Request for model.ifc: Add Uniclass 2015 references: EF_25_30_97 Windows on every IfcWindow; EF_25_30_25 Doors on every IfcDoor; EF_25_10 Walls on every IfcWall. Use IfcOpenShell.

First a look at what the model holds.

```python
import ifcopenshell

model = ifcopenshell.open("model.ifc")
print(model.schema)
print("classifications:", [c.Name for c in model.by_type("IfcClassification")])
for ifc_class in ("IfcDoor", "IfcRoof", "IfcStair", "IfcWall", "IfcWindow"):
    print(ifc_class, len(model.by_type(ifc_class)))
```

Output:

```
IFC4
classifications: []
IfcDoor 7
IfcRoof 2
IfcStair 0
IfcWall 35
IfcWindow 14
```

```python
import ifcopenshell
import ifcopenshell.api.classification

model = ifcopenshell.open("model.ifc")

system = ifcopenshell.api.classification.add_classification(model, classification="Uniclass 2015")

codes = {
    "IfcWindow": ("EF_25_30_97", "Windows"),
    "IfcDoor": ("EF_25_30_25", "Doors"),
    "IfcWall": ("EF_25_10", "Walls"),
}
for ifc_class, (code, name) in codes.items():
    products = model.by_type(ifc_class)
    ifcopenshell.api.classification.add_reference(
        model, products=products, classification=system, identification=code, name=name
    )
    print(code, len(products))

model.write("model_rev.ifc")
```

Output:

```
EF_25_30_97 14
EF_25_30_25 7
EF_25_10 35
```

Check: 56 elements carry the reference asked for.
